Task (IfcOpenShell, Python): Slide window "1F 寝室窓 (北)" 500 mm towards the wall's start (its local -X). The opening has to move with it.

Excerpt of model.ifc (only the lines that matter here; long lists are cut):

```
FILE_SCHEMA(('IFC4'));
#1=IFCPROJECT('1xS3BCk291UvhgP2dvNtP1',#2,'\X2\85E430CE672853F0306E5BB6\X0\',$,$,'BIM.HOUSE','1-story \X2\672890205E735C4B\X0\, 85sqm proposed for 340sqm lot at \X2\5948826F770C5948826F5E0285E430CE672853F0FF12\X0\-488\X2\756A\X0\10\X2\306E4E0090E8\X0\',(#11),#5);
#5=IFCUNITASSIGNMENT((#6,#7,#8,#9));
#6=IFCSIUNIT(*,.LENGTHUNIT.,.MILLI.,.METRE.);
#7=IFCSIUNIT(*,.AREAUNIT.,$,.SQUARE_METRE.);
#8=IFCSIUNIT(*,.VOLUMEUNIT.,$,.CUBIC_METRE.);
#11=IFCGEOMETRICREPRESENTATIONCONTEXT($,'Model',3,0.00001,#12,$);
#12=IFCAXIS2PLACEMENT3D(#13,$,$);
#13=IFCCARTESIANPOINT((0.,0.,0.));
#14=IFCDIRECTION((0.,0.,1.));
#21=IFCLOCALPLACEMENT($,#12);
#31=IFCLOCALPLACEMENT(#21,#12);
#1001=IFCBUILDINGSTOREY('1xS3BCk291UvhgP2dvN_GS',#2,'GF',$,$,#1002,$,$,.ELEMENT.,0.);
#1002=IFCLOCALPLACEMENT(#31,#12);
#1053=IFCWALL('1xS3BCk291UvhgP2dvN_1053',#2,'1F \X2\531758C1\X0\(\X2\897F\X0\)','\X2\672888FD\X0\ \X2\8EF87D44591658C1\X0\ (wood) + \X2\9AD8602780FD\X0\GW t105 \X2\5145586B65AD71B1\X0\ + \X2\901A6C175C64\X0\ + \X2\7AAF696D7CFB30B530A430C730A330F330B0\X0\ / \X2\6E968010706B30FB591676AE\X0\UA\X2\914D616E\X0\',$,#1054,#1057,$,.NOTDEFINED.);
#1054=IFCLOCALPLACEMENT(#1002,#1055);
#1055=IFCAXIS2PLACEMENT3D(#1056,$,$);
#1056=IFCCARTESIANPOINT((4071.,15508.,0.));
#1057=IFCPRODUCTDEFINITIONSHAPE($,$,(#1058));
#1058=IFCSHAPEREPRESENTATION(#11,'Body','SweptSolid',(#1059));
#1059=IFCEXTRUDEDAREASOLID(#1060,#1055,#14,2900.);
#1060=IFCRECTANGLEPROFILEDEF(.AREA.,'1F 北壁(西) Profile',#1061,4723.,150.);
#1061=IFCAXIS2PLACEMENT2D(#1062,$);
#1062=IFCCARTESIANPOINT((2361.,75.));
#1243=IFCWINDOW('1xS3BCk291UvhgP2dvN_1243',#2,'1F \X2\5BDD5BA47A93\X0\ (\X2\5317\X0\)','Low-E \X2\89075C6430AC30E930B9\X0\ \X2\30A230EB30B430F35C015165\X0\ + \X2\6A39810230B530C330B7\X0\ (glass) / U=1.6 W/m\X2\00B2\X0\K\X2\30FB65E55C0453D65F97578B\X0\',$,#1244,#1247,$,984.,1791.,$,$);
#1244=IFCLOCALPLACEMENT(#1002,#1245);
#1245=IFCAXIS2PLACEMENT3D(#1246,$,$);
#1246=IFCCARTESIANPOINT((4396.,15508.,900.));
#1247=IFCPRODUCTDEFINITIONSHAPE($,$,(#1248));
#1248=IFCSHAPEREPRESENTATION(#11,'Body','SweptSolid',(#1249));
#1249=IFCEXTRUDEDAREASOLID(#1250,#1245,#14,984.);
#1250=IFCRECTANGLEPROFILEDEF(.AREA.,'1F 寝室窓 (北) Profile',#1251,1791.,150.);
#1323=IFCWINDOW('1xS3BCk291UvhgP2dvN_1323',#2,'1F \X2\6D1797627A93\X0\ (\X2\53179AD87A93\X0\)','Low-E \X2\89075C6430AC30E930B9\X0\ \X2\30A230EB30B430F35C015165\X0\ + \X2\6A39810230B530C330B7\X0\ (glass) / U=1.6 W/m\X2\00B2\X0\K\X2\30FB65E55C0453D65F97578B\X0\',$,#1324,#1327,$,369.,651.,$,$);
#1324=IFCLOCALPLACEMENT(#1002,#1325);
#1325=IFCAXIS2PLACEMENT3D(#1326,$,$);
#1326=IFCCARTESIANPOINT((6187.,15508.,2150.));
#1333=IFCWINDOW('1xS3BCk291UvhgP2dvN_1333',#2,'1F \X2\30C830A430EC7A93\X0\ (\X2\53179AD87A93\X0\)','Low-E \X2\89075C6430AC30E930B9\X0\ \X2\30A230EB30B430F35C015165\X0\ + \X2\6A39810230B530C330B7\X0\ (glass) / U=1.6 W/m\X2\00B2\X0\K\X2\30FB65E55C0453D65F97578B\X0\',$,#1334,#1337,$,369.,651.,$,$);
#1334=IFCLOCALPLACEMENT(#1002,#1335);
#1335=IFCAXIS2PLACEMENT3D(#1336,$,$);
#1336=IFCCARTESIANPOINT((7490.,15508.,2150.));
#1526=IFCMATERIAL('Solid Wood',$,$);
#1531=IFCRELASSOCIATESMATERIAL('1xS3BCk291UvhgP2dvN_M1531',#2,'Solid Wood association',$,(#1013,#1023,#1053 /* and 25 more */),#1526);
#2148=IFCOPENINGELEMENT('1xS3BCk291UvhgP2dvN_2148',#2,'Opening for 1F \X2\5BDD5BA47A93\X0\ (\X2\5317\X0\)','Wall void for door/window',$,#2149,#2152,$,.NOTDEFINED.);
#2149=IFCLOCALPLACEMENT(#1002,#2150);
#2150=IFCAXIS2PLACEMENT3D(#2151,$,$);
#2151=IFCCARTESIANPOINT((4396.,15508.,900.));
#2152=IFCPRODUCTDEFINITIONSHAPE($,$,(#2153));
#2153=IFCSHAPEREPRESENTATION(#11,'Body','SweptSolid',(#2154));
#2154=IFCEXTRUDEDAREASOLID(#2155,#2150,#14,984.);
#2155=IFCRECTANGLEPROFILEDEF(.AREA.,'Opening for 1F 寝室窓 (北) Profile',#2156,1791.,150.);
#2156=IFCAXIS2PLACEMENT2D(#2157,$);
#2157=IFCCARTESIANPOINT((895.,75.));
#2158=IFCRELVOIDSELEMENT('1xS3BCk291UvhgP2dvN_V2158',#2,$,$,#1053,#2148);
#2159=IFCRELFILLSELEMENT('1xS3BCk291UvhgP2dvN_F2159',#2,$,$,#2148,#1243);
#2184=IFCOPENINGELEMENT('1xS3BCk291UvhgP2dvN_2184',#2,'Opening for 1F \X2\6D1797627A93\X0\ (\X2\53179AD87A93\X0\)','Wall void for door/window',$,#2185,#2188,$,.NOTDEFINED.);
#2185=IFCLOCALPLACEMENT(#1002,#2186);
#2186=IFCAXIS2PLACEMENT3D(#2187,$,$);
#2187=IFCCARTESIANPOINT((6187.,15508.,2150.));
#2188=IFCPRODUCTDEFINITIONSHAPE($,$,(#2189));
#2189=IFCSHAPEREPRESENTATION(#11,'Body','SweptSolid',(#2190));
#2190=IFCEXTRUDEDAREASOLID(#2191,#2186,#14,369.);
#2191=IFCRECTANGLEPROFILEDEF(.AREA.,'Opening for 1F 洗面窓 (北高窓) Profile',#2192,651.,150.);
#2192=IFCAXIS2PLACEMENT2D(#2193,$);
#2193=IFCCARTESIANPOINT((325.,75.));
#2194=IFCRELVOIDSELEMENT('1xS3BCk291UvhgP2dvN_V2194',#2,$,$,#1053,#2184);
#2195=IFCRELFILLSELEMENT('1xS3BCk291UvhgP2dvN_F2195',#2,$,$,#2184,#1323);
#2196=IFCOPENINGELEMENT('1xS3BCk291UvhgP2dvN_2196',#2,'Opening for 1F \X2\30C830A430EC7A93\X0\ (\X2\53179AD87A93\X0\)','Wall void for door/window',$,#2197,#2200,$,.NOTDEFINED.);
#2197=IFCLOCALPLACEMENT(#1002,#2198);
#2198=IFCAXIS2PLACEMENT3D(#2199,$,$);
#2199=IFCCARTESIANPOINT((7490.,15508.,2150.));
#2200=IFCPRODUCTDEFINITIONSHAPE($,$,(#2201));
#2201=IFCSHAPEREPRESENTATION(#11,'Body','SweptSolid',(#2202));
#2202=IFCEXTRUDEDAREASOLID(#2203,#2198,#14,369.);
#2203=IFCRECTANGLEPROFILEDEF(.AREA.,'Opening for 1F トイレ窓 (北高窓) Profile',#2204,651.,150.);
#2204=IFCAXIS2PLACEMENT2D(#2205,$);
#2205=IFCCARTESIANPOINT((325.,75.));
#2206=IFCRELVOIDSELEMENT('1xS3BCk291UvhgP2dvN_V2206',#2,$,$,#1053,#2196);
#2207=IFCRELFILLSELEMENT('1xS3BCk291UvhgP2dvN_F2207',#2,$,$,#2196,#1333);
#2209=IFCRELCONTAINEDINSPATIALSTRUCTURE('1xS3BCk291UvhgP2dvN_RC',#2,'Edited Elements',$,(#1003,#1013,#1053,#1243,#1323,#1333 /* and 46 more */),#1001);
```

```python
import ifcopenshell
import ifcopenshell.api.geometry
import ifcopenshell.util.placement
import ifcopenshell.util.unit

model = ifcopenshell.open("model.ifc")
unit_scale = ifcopenshell.util.unit.calculate_unit_scale(model)

window = model.by_id(1243)
opening = window.FillsVoids[0].RelatingOpeningElement
wall = opening.VoidsElements[0].RelatingBuildingElement

wall_matrix = ifcopenshell.util.placement.get_local_placement(wall.ObjectPlacement)
shift = wall_matrix[:3, 0] * -0.5 / unit_scale
before = ifcopenshell.util.placement.get_local_placement(window.ObjectPlacement)[:3, 3].copy()

# The window is not placed relative to its opening, so move both.
for product in (opening, window):
    matrix = ifcopenshell.util.placement.get_local_placement(product.ObjectPlacement)
    matrix[:3, 3] += shift
    ifcopenshell.api.geometry.edit_object_placement(model, product=product, matrix=matrix, is_si=False)

after = ifcopenshell.util.placement.get_local_placement(window.ObjectPlacement)[:3, 3]
print("window moved by", (after - before).round(3) + 0.0)

model.write("model_edited.ifc")
```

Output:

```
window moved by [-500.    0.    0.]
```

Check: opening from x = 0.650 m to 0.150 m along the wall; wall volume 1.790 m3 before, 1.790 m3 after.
